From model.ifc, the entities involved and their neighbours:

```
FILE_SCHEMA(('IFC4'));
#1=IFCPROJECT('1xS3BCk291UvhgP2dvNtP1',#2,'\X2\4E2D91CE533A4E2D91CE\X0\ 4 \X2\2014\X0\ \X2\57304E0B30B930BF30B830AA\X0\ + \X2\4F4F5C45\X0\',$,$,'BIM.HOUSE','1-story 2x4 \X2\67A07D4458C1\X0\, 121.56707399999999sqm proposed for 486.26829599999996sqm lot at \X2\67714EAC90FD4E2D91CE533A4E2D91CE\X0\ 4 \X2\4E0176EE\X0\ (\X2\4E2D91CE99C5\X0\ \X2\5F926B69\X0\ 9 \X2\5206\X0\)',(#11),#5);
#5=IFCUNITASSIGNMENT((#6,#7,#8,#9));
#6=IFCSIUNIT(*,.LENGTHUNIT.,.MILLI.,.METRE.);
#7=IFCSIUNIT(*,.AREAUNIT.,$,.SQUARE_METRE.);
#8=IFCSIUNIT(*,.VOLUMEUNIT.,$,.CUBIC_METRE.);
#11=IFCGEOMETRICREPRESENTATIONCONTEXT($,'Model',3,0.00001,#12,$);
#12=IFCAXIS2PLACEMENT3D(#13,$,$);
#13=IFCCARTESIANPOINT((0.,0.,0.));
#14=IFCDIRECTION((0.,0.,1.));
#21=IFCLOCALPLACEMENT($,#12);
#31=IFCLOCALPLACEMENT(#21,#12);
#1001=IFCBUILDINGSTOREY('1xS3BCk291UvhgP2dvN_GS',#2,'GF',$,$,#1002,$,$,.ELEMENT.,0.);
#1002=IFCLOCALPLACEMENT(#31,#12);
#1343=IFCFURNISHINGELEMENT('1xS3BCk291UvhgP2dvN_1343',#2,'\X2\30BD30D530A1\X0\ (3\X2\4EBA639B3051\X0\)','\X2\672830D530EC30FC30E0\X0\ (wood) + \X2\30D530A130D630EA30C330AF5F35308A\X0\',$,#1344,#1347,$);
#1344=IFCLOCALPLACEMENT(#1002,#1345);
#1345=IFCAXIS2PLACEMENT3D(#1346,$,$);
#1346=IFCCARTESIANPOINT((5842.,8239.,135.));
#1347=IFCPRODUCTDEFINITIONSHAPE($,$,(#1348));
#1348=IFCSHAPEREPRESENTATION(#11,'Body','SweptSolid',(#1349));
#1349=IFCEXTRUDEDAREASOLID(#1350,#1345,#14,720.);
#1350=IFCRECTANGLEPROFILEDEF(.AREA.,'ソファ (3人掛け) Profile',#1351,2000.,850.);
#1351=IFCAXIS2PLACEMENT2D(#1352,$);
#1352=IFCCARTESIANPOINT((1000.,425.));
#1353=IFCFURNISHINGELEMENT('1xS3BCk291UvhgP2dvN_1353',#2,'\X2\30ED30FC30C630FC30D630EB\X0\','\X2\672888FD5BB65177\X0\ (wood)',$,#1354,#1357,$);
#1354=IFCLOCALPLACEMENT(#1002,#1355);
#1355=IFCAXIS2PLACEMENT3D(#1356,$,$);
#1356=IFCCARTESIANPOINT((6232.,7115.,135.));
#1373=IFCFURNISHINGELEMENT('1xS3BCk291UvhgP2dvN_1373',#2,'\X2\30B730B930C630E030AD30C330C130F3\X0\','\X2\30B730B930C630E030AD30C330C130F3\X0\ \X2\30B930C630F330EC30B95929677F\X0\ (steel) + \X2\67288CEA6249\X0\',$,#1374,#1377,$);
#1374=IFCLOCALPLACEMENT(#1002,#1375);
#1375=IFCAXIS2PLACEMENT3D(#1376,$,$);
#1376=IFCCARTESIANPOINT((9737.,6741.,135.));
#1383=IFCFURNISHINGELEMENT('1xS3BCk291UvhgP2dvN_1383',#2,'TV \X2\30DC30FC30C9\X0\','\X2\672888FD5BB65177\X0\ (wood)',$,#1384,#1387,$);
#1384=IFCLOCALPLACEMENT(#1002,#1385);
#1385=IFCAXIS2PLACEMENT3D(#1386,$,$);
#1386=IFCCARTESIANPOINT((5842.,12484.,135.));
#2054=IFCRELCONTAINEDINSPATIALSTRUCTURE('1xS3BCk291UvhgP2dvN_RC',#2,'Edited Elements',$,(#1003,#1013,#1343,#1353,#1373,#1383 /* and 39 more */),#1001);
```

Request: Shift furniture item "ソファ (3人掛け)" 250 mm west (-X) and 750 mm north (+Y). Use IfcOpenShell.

```python
import ifcopenshell
import ifcopenshell.api.geometry
import ifcopenshell.util.placement
import ifcopenshell.util.unit

model = ifcopenshell.open("model.ifc")
unit_scale = ifcopenshell.util.unit.calculate_unit_scale(model)

item = model.by_guid("1xS3BCk291UvhgP2dvN_1343")
matrix = ifcopenshell.util.placement.get_local_placement(item.ObjectPlacement)
matrix[0, 3] -= 0.25 / unit_scale
matrix[1, 3] += 0.75 / unit_scale
ifcopenshell.api.geometry.edit_object_placement(model, product=item, matrix=matrix, is_si=False)

print(ifcopenshell.util.placement.get_local_placement(item.ObjectPlacement).round(3) + 0.0)

model.write("model-out.ifc")
```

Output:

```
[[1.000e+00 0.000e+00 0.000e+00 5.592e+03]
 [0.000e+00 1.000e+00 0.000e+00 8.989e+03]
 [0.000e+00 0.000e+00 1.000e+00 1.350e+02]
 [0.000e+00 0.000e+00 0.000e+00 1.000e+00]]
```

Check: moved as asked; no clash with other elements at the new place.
